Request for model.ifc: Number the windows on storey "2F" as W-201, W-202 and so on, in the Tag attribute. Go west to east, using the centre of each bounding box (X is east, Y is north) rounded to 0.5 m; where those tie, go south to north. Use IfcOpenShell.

First a look at what the model holds.

```python
import ifcopenshell
import ifcopenshell.util.element
import ifcopenshell.util.placement

model = ifcopenshell.open("model.ifc")
print(model.schema)
storey = next(s for s in model.by_type("IfcBuildingStorey") if s.Name == "2F")
windows = [e for e in ifcopenshell.util.element.get_decomposition(storey) if e.is_a("IfcWindow")]
for e in sorted(windows, key=lambda e: e.id()):
    origin = ifcopenshell.util.placement.get_local_placement(e.ObjectPlacement)[:3, 3]
    print(e.id(), e.Tag, e.Name, origin.round(2) + 0.0, sep=" | ")
```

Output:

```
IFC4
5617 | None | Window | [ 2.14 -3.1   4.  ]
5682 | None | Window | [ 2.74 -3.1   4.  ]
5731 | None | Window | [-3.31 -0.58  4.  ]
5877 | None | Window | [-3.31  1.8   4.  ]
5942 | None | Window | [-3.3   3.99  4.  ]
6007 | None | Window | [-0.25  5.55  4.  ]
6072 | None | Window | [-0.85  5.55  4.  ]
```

```python
import ifcopenshell
import ifcopenshell.geom
import ifcopenshell.util.element
import ifcopenshell.util.shape

model = ifcopenshell.open("model.ifc")
settings = ifcopenshell.geom.settings()
settings.set("use-world-coords", True)


def centre(element):
    shape = ifcopenshell.geom.create_shape(settings, element)
    return ifcopenshell.util.shape.get_bbox_centroid(shape.geometry)


storey = next(s for s in model.by_type("IfcBuildingStorey") if s.Name == "2F")
windows = [e for e in ifcopenshell.util.element.get_decomposition(storey) if e.is_a("IfcWindow")]

# Insertion points can sit at a corner or the storey origin, so sort by the geometry (in metres).
centres = {e: centre(e) for e in windows}
windows.sort(key=lambda e: (round(centres[e][0] / 0.5), centres[e][1]))

for i, e in enumerate(windows, start=1):
    number = f"W-2{i:02d}"
    e.Tag = number
    print(e.id(), number)

model.write("model_edited.ifc")
```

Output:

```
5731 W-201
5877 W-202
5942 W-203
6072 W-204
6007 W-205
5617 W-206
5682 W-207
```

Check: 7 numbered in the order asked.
